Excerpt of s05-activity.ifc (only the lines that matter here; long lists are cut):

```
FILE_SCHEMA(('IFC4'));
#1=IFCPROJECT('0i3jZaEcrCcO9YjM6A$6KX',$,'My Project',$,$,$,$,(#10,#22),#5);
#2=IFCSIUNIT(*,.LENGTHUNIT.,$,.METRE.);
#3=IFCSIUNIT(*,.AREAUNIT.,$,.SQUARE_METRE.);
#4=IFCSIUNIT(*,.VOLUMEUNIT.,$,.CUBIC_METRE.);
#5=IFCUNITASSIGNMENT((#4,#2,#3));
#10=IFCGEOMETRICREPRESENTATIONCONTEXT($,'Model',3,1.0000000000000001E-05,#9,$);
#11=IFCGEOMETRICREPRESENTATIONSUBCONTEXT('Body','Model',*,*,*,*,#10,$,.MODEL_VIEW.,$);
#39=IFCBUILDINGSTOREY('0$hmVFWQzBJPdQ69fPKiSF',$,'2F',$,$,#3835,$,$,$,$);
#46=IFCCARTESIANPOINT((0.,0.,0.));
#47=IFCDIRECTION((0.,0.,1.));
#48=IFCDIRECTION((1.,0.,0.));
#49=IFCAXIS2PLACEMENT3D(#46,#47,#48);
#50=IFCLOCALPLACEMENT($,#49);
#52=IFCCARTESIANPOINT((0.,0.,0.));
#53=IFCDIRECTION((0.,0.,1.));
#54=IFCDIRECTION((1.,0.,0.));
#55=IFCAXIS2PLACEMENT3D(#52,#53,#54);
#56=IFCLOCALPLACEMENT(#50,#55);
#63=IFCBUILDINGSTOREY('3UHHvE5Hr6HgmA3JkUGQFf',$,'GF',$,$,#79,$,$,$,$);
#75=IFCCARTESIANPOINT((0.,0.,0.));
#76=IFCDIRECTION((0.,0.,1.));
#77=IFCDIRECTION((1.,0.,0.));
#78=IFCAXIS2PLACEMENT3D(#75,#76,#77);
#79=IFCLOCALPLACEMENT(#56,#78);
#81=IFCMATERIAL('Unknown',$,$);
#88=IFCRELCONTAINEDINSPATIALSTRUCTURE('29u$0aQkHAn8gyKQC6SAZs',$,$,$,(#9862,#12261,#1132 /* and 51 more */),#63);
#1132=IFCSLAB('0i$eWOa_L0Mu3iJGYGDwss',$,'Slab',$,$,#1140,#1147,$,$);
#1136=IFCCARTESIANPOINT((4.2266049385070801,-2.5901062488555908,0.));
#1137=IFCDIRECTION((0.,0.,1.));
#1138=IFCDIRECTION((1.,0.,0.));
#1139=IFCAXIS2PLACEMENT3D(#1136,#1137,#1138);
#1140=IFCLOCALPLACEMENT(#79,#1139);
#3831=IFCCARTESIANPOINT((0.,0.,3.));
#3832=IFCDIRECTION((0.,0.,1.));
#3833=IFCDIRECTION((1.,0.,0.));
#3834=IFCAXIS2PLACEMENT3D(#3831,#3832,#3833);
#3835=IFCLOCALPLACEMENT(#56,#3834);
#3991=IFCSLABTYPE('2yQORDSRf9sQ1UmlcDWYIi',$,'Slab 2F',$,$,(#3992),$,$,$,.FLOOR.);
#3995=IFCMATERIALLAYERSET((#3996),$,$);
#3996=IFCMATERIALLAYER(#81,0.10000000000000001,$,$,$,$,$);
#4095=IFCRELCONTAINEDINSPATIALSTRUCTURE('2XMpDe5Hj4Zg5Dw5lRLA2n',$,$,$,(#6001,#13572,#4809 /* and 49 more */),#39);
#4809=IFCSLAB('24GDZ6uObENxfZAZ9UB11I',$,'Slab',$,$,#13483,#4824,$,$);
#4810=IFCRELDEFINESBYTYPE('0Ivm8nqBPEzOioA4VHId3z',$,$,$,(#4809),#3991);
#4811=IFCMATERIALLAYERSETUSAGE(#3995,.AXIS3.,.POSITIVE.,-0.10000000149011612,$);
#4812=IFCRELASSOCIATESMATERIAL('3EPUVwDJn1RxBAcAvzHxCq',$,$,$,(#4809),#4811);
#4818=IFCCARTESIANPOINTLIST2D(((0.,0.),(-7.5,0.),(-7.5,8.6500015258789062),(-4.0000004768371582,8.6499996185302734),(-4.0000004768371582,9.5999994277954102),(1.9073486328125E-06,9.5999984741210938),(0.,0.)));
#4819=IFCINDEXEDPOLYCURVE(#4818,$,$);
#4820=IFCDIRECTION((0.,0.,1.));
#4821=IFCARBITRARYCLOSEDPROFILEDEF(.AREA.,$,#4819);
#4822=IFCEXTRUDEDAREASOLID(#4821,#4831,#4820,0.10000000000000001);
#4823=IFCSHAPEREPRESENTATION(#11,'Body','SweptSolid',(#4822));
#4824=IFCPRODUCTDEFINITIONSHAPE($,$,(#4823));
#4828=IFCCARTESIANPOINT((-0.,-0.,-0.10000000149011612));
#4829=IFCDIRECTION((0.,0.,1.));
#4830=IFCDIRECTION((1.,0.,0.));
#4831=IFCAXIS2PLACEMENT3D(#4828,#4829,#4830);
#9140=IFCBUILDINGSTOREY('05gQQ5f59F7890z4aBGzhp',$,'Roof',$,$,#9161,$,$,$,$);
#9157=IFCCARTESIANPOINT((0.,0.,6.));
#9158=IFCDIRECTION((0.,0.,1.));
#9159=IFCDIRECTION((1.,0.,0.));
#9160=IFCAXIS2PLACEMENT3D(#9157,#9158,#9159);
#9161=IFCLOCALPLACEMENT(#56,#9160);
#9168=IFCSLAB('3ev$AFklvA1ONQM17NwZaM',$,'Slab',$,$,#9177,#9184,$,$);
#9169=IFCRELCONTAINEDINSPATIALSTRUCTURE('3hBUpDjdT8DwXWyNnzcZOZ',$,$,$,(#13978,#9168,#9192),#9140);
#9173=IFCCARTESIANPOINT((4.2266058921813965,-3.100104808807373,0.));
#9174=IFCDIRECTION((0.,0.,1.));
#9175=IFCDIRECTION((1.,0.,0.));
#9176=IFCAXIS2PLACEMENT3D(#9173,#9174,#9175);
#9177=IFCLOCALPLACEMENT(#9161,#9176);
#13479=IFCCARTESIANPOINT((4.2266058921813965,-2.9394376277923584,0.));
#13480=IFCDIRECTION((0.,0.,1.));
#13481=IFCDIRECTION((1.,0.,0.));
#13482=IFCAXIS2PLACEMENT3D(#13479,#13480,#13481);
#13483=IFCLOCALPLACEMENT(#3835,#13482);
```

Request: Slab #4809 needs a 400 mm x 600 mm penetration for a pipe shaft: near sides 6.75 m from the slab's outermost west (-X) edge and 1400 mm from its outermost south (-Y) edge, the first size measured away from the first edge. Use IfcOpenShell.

```python
import numpy as np
import ifcopenshell
import ifcopenshell.api.feature
import ifcopenshell.api.geometry
import ifcopenshell.api.root
import ifcopenshell.geom
import ifcopenshell.util.placement
import ifcopenshell.util.representation
import ifcopenshell.util.shape
import ifcopenshell.util.unit

model = ifcopenshell.open("s05-activity.ifc")
unit_scale = ifcopenshell.util.unit.calculate_unit_scale(model)
settings = ifcopenshell.geom.settings()


def volume(element):
    """Net volume in cubic metres, openings subtracted."""
    shape = ifcopenshell.geom.create_shape(settings, element)
    return ifcopenshell.util.shape.get_volume(shape.geometry)


slab = model.by_id(4809)
before = volume(slab)

# Extent in the slab's own axes, in metres. The edges named are its -X and -Y sides.
slab_shape = ifcopenshell.geom.create_shape(settings, slab)
vertices = ifcopenshell.util.shape.get_vertices(slab_shape.geometry)
x_min, y_min, bottom = vertices.min(axis=0)
top = vertices[:, 2].max()

opening = ifcopenshell.api.root.create_entity(model, ifc_class="IfcOpeningElement", name="Pipe shaft opening", predefined_type="OPENING")
context = ifcopenshell.util.representation.get_context(model, "Model", "Body", "MODEL_VIEW")
width, depth = 0.4, 0.6
outline = [(0.0, 0.0), (width, 0.0), (width, depth), (0.0, depth), (0.0, 0.0)]
# Overshoot both faces by 50 mm so the cut is clean.
shape = ifcopenshell.api.geometry.add_slab_representation(
    model, context=context, depth=top - bottom + 0.1, polyline=outline
)
ifcopenshell.api.geometry.assign_representation(model, product=opening, representation=shape)

matrix = ifcopenshell.util.placement.get_local_placement(slab.ObjectPlacement)
matrix[:, 3] = matrix @ np.append(np.array([x_min + 6.75, y_min + 1.4, bottom - 0.05]) / unit_scale, 1.0)
ifcopenshell.api.geometry.edit_object_placement(model, product=opening, matrix=matrix, is_si=False)
ifcopenshell.api.feature.add_feature(model, feature=opening, element=slab)

after = volume(slab)

print(f"slab volume {before:.3f} -> {after:.3f} m3")

model.write("s05-activity_v2.ifc")
```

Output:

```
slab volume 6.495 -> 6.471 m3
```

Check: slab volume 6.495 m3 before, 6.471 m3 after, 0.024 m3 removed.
